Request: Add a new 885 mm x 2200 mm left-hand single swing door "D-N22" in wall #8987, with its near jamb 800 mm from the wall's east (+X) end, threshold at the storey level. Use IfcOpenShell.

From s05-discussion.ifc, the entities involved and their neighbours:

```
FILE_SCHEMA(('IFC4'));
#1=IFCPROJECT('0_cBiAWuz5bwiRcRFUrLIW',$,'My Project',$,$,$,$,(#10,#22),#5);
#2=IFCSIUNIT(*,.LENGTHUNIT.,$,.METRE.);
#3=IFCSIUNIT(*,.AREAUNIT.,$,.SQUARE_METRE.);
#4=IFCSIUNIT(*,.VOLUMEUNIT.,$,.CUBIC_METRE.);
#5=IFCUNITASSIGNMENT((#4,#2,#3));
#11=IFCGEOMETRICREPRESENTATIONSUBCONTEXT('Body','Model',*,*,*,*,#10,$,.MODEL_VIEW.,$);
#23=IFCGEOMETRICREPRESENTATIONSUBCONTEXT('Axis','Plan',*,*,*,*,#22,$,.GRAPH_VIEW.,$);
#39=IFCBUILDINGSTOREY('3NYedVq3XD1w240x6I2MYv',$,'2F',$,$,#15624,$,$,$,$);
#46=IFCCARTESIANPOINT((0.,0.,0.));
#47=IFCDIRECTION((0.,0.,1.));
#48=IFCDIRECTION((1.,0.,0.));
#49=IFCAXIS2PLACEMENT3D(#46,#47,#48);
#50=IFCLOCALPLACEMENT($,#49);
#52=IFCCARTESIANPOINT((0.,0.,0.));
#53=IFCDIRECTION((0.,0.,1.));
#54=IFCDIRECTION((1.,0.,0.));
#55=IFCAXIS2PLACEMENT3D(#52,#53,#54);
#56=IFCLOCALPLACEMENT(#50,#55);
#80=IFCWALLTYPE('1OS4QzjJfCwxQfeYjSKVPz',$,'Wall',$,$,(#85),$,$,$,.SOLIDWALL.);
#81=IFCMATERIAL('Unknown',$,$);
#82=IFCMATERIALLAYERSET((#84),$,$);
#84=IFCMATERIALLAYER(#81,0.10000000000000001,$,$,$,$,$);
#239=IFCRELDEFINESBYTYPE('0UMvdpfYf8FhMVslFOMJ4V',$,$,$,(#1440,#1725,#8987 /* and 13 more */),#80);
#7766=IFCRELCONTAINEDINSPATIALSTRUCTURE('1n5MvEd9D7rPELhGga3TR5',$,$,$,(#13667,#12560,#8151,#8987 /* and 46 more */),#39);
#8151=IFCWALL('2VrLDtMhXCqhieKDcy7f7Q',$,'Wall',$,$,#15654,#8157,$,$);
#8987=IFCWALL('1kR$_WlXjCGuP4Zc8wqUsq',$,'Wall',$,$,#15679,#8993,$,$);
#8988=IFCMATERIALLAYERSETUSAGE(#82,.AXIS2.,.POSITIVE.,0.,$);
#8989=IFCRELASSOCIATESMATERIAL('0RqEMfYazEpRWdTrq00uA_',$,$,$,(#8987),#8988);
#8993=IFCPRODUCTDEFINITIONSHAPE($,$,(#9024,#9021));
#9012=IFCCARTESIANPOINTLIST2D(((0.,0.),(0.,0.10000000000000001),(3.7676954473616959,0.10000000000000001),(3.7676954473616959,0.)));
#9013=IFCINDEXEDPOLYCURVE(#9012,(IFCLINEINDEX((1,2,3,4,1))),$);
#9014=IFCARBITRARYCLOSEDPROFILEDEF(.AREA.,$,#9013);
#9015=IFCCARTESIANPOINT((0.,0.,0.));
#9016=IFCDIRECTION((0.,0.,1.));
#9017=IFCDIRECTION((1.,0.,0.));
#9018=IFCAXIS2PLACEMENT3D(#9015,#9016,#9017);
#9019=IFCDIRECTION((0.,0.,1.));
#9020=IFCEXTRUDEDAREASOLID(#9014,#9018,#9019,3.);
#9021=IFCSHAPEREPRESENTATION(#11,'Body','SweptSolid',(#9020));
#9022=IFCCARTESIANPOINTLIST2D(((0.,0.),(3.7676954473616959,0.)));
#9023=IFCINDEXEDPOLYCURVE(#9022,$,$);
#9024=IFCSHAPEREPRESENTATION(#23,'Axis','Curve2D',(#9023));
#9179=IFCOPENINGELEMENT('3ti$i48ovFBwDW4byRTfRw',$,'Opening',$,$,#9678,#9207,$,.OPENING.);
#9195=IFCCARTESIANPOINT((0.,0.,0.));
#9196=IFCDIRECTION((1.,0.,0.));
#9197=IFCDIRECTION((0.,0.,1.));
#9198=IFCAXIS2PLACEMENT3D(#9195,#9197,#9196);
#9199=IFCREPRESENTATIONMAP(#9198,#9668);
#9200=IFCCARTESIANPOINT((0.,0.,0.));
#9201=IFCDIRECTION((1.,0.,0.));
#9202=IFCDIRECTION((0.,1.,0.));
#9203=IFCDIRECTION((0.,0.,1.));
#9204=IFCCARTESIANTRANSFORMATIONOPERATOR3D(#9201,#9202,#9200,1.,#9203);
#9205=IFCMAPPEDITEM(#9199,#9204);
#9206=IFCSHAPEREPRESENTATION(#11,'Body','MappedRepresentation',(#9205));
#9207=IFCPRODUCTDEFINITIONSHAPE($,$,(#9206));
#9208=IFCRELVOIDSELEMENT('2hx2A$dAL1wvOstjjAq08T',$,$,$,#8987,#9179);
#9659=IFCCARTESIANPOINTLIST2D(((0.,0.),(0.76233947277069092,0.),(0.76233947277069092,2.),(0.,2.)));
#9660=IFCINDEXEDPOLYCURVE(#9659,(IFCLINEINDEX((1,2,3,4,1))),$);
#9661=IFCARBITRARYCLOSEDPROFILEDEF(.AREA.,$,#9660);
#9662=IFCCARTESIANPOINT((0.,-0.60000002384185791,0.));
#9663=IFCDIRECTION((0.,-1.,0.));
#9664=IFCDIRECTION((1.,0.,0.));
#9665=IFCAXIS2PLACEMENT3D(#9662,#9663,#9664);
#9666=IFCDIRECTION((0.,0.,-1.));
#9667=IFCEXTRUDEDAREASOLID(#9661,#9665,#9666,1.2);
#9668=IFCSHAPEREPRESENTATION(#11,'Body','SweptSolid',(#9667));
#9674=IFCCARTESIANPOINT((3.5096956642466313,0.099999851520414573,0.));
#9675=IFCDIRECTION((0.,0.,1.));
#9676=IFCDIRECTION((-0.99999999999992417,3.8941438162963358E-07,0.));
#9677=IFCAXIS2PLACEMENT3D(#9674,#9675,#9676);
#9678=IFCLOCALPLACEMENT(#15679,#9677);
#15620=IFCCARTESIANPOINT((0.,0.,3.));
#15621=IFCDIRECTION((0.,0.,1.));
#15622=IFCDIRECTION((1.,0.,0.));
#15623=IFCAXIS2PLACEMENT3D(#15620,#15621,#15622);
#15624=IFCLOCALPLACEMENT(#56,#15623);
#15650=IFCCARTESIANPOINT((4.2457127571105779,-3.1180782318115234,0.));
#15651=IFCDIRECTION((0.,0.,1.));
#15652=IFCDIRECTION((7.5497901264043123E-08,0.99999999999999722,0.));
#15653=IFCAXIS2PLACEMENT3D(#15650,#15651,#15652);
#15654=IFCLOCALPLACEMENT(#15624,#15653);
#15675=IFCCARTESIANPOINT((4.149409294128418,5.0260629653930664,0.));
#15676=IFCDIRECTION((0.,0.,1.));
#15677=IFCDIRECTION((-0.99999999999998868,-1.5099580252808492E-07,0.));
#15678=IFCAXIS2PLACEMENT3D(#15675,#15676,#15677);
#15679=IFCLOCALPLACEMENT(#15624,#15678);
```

```python
import numpy as np
import ifcopenshell
import ifcopenshell.api.feature
import ifcopenshell.api.geometry
import ifcopenshell.api.root
import ifcopenshell.api.spatial
import ifcopenshell.geom
import ifcopenshell.util.element
import ifcopenshell.util.placement
import ifcopenshell.util.representation
import ifcopenshell.util.shape
import ifcopenshell.util.unit

model = ifcopenshell.open("s05-discussion.ifc")
unit_scale = ifcopenshell.util.unit.calculate_unit_scale(model)
settings = ifcopenshell.geom.settings()


def volume(element):
    """Net volume in cubic metres, openings subtracted."""
    shape = ifcopenshell.geom.create_shape(settings, element)
    return ifcopenshell.util.shape.get_volume(shape.geometry)


wall = model.by_guid("1kR$_WlXjCGuP4Zc8wqUsq")
storey = ifcopenshell.util.element.get_container(wall, ifc_class="IfcBuildingStorey")
context = ifcopenshell.util.representation.get_context(model, "Model", "Body", "MODEL_VIEW")
before = volume(wall)

width, height, from_end, sill = 0.885, 2.2, 0.8, 0.0  # metres

# The wall runs along its own X axis, and the end named is its -X end.
wall_shape = ifcopenshell.geom.create_shape(settings, wall)
x, y, z = ifcopenshell.util.shape.get_vertices(wall_shape.geometry).T
start = x.min() + from_end
face, thickness = float(y.min()), float(y.max() - y.min())
wall_matrix = ifcopenshell.util.placement.get_local_placement(wall.ObjectPlacement)
level = ifcopenshell.util.placement.get_local_placement(storey.ObjectPlacement)[2, 3]


def in_wall(x, y):
    """Placement at x, y metres in the wall's axes, at sill height."""
    matrix = wall_matrix.copy()
    matrix[:, 3] = wall_matrix @ np.array([x / unit_scale, y / unit_scale, 0.0, 1.0])
    matrix[2, 3] = level + sill / unit_scale
    return matrix


# Opening: a box that overshoots both wall faces by 50 mm.
opening = ifcopenshell.api.root.create_entity(model, ifc_class="IfcOpeningElement", predefined_type="OPENING")
box = ifcopenshell.api.geometry.add_wall_representation(
    model, context=context, length=width, height=height, thickness=thickness + 0.1
)
ifcopenshell.api.geometry.assign_representation(model, product=opening, representation=box)
ifcopenshell.api.geometry.edit_object_placement(model, product=opening, matrix=in_wall(start, face - 0.05), is_si=False)
ifcopenshell.api.feature.add_feature(model, feature=opening, element=wall)

door = ifcopenshell.api.root.create_entity(model, ifc_class="IfcDoor", name="D-N22", predefined_type="DOOR")
door.OverallWidth, door.OverallHeight = width / unit_scale, height / unit_scale
door.OperationType = "SINGLE_SWING_LEFT"
body = ifcopenshell.api.geometry.add_door_representation(
    model,
    context=context,
    overall_width=door.OverallWidth,
    overall_height=door.OverallHeight,
    operation_type="SINGLE_SWING_LEFT",
    lining_properties={"LiningDepth": thickness / unit_scale, "ThresholdDepth": thickness / unit_scale},
)
ifcopenshell.api.geometry.assign_representation(model, product=door, representation=body)
ifcopenshell.api.spatial.assign_container(model, products=[door], relating_structure=storey)
ifcopenshell.api.feature.add_filling(model, opening=opening, element=door)

# The lining spans the wall, so the door starts at the wall face.
ifcopenshell.api.geometry.edit_object_placement(model, product=door, matrix=in_wall(start, face), is_si=False)

after = volume(wall)

print(f"wall volume {before:.3f} -> {after:.3f} m3")

model.write("s05-discussion_v2.ifc")
```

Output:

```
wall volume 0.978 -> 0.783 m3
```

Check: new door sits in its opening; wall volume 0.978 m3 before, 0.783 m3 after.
